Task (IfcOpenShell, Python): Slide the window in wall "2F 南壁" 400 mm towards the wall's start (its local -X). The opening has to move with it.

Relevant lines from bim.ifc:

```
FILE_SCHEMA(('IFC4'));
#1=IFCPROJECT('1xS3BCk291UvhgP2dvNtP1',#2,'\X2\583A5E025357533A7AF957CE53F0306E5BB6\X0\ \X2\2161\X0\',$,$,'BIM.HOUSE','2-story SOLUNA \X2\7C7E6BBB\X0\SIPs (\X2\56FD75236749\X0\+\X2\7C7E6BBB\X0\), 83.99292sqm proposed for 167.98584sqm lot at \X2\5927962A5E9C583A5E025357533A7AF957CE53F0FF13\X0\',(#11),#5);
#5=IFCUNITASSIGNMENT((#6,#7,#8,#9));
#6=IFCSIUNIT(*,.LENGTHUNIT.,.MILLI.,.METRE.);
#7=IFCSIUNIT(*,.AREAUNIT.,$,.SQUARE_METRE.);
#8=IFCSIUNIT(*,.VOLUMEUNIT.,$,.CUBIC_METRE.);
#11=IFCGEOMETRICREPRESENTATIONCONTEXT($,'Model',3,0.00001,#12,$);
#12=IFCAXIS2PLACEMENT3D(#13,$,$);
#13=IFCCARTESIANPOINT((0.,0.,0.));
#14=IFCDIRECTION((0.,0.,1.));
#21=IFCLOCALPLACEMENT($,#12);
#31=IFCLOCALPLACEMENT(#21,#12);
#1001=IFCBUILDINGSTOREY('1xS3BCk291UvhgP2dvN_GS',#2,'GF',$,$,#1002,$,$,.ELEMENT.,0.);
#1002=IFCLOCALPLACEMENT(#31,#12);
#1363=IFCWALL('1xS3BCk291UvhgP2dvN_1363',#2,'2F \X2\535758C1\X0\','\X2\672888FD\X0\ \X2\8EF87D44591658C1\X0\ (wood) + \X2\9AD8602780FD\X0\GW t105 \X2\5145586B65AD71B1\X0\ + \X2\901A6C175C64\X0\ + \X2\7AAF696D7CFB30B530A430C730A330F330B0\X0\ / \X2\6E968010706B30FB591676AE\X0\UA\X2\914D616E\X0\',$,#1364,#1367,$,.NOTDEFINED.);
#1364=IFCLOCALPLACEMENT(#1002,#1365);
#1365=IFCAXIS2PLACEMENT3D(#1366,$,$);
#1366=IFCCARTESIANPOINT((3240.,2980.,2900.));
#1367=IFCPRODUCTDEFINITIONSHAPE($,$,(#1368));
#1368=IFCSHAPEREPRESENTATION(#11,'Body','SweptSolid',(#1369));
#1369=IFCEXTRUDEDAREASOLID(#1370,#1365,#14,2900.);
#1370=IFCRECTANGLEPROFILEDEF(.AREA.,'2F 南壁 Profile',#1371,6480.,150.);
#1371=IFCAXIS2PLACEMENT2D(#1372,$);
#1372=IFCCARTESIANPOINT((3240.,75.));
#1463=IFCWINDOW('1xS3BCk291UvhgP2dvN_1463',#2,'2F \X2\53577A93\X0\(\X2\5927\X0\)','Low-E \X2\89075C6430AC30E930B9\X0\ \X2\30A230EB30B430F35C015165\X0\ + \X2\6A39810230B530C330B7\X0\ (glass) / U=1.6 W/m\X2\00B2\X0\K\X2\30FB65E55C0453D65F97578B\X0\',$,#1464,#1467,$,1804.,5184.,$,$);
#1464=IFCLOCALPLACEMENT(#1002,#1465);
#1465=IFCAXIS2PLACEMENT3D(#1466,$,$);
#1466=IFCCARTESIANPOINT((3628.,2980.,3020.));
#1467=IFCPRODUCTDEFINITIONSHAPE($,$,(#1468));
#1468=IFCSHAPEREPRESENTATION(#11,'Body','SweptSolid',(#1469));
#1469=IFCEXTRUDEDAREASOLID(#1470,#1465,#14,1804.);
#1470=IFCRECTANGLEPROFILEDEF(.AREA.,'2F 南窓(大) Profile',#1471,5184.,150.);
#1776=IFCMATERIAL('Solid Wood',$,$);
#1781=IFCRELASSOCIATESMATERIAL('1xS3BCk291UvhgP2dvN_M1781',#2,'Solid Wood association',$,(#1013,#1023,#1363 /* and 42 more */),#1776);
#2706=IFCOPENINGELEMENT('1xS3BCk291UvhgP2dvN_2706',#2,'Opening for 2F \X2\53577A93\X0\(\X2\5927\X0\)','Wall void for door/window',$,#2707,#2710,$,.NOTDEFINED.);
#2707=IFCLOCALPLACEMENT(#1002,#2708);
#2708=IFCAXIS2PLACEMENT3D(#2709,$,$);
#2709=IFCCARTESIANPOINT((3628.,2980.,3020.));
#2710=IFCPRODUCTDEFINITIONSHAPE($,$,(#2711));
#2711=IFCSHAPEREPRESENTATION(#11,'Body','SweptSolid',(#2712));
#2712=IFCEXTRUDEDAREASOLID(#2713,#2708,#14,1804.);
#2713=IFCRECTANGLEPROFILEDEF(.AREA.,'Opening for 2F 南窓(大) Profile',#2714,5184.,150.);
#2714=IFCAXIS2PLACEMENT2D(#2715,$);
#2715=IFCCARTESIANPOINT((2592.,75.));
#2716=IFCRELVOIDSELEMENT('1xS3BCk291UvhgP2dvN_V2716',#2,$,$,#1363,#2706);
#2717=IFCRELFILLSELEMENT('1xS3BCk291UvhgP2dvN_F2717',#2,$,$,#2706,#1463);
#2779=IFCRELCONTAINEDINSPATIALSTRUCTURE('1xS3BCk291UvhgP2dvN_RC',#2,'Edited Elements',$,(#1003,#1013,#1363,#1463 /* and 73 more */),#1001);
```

```python
import ifcopenshell
import ifcopenshell.api.geometry
import ifcopenshell.util.placement

model = ifcopenshell.open("bim.ifc")

window = model.by_guid("1xS3BCk291UvhgP2dvN_1463")
opening = window.FillsVoids[0].RelatingOpeningElement
wall = opening.VoidsElements[0].RelatingBuildingElement

wall_matrix = ifcopenshell.util.placement.get_local_placement(wall.ObjectPlacement)
shift = wall_matrix[:3, 0] * -400.0
before = ifcopenshell.util.placement.get_local_placement(window.ObjectPlacement)[:3, 3].copy()

# The window is not placed relative to its opening, so move both.
for product in (opening, window):
    matrix = ifcopenshell.util.placement.get_local_placement(product.ObjectPlacement)
    matrix[:3, 3] += shift
    ifcopenshell.api.geometry.edit_object_placement(model, product=product, matrix=matrix, is_si=False)

after = ifcopenshell.util.placement.get_local_placement(window.ObjectPlacement)[:3, 3]
print("window moved by", (after - before).round(3) + 0.0)

model.write("bim_rev.ifc")
```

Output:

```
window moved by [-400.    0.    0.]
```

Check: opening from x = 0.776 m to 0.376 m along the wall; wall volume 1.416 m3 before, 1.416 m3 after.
